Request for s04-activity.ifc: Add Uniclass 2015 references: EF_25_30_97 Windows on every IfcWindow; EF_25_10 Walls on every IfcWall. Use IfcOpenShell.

First a look at what the model holds.

```python
import ifcopenshell

model = ifcopenshell.open("s04-activity.ifc")
print(model.schema)
print("classifications:", [c.Name for c in model.by_type("IfcClassification")])
for ifc_class in ("IfcDoor", "IfcRoof", "IfcStair", "IfcWall", "IfcWindow"):
    print(ifc_class, len(model.by_type(ifc_class)))
```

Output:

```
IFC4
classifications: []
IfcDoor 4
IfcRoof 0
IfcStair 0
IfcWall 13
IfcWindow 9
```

```python
import ifcopenshell
import ifcopenshell.api.classification

model = ifcopenshell.open("s04-activity.ifc")

system = ifcopenshell.api.classification.add_classification(model, classification="Uniclass 2015")

codes = {
    "IfcWindow": ("EF_25_30_97", "Windows"),
    "IfcWall": ("EF_25_10", "Walls"),
}
for ifc_class, (code, name) in codes.items():
    products = model.by_type(ifc_class)
    ifcopenshell.api.classification.add_reference(
        model, products=products, classification=system, identification=code, name=name
    )
    print(code, len(products))

model.write("s04-activity_rev.ifc")
```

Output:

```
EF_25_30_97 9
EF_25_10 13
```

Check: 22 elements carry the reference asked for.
